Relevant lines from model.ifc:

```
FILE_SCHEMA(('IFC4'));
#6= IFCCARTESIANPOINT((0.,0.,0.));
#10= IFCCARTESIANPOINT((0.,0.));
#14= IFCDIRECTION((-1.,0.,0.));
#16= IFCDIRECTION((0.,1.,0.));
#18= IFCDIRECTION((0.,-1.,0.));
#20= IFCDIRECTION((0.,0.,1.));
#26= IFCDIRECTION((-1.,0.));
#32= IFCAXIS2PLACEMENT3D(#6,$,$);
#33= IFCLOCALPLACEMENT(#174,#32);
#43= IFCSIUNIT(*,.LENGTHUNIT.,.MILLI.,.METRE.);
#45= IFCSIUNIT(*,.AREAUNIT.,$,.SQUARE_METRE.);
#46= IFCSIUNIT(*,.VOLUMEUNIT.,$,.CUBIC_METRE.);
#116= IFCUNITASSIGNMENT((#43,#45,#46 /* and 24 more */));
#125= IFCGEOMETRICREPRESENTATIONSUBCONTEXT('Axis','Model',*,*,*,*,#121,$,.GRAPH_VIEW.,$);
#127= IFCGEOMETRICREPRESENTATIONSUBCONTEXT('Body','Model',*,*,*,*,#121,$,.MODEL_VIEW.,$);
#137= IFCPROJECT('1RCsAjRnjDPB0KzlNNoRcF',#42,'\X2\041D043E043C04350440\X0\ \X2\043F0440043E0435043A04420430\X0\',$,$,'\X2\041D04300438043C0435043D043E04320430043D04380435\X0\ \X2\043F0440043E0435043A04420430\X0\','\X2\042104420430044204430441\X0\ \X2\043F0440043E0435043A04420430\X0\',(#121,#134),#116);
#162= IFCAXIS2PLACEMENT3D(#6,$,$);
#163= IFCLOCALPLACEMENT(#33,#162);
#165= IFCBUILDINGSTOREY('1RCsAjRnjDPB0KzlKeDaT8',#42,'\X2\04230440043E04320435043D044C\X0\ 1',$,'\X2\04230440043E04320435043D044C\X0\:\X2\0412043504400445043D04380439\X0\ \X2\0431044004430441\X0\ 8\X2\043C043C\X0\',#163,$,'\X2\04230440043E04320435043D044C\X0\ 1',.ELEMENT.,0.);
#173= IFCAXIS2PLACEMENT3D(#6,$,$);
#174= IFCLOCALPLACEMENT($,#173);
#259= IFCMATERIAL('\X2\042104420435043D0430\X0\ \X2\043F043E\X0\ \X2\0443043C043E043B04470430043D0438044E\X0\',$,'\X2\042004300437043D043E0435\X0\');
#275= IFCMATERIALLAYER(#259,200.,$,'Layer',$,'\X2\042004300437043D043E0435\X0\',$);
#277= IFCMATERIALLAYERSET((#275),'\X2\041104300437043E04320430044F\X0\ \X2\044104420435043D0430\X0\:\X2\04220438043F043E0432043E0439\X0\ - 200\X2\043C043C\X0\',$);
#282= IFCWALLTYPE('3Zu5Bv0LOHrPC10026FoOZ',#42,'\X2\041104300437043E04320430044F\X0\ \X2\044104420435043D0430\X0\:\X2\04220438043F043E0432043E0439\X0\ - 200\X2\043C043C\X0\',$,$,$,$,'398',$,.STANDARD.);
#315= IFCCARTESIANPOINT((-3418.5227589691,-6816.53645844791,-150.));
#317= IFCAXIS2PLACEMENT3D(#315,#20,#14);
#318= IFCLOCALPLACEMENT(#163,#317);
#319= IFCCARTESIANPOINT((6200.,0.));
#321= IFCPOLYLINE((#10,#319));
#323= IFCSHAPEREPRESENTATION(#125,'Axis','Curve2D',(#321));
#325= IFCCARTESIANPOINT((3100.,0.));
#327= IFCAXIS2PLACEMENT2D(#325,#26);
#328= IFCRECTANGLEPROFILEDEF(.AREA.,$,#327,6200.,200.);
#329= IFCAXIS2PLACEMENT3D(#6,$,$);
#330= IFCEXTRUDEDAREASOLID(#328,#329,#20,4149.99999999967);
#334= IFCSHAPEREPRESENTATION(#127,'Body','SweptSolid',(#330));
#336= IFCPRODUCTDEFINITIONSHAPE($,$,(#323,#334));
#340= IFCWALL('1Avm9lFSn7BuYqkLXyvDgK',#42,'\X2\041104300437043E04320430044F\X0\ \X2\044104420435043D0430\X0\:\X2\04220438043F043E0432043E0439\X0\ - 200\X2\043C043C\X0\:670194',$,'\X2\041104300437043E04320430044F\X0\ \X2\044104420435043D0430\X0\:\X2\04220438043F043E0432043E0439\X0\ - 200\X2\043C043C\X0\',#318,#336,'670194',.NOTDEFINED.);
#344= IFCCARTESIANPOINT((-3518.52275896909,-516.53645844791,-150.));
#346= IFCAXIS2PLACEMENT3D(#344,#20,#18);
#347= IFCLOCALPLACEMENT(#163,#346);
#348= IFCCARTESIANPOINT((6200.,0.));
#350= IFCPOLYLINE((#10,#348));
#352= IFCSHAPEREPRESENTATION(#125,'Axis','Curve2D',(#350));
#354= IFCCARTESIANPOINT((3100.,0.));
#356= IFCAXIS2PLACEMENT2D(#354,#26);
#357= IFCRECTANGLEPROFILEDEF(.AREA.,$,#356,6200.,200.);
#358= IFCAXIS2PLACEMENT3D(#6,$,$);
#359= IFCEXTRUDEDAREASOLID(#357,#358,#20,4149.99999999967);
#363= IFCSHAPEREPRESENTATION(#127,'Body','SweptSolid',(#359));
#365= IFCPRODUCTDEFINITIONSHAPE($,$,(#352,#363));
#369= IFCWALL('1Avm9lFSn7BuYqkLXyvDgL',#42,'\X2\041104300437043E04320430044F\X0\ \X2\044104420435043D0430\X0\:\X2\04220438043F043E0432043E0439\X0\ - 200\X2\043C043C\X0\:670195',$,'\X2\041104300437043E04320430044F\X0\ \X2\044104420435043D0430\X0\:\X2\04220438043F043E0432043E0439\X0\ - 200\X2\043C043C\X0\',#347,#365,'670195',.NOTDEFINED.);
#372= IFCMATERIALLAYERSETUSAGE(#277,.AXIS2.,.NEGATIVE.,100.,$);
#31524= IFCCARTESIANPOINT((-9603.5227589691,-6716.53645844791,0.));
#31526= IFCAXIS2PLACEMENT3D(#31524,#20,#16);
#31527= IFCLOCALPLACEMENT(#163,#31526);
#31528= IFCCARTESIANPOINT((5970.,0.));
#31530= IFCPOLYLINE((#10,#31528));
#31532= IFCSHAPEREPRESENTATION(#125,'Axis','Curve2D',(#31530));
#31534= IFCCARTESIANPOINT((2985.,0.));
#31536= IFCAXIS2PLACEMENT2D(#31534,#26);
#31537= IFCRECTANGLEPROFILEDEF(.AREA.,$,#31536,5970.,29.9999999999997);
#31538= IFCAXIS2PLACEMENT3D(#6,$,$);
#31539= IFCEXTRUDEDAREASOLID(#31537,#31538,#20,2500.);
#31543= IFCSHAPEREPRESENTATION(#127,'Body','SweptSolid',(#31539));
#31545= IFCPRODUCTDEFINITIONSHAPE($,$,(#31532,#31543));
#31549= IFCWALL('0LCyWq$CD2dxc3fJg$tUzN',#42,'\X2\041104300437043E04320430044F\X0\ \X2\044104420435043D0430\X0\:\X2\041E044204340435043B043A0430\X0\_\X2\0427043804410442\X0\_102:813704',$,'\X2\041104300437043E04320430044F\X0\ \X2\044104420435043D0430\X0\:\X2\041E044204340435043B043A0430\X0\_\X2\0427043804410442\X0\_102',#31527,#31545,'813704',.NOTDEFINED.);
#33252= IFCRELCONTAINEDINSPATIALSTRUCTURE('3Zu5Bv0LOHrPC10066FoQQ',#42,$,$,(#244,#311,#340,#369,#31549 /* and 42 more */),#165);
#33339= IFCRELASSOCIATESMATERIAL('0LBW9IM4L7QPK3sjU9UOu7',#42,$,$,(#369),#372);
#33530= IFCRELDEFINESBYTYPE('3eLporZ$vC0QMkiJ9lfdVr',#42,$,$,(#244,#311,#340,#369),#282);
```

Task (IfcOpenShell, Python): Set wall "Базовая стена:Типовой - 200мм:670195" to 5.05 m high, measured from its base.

```python
import ifcopenshell
import ifcopenshell.geom
import ifcopenshell.util.representation
import ifcopenshell.util.shape
import ifcopenshell.util.unit

model = ifcopenshell.open("model.ifc")
unit_scale = ifcopenshell.util.unit.calculate_unit_scale(model)
settings = ifcopenshell.geom.settings()


def volume(element):
    """Net volume in cubic metres, openings subtracted."""
    shape = ifcopenshell.geom.create_shape(settings, element)
    return ifcopenshell.util.shape.get_volume(shape.geometry)


wall = model.by_guid("1Avm9lFSn7BuYqkLXyvDgL")
before = volume(wall)

body = ifcopenshell.util.representation.get_representation(wall, "Model", "Body")
solid = body.Items[0]
old_height = solid.Depth
solid.Depth = 5.05 / unit_scale
after = volume(wall)

print(f"height {old_height:g} -> {solid.Depth:g}, volume {before:.3f} -> {after:.3f} m3")

model.write("model_rev.ifc")
```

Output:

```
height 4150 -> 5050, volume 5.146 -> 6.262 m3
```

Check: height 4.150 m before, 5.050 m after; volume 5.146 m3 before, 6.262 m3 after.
